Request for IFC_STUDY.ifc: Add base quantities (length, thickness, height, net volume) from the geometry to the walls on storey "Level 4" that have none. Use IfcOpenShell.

First a look at what the model holds.

```python
import ifcopenshell
import ifcopenshell.util.element
import ifcopenshell.util.unit

model = ifcopenshell.open("IFC_STUDY.ifc")
print(model.schema)
for unit_type in ("LENGTHUNIT", "AREAUNIT", "VOLUMEUNIT"):
    print(unit_type, ifcopenshell.util.unit.calculate_unit_scale(model, unit_type))
storey = next(s for s in model.by_type("IfcBuildingStorey") if s.Name == "Level 4")
walls = [e for e in ifcopenshell.util.element.get_decomposition(storey) if e.is_a("IfcWall")]
for e in sorted(walls, key=lambda e: e.id()):
    print(e.id(), e.is_a(), e.Name, list(ifcopenshell.util.element.get_psets(e, qtos_only=True)), sep=" | ")
```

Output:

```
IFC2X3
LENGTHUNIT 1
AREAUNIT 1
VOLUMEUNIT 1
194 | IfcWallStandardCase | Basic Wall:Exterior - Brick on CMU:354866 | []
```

```python
import ifcopenshell
import ifcopenshell.api.pset
import ifcopenshell.geom
import ifcopenshell.util.element
import ifcopenshell.util.shape
import ifcopenshell.util.unit

model = ifcopenshell.open("IFC_STUDY.ifc")
unit_scale = ifcopenshell.util.unit.calculate_unit_scale(model)
volume_scale = ifcopenshell.util.unit.calculate_unit_scale(model, "VOLUMEUNIT")
settings = ifcopenshell.geom.settings()

storey = next(s for s in model.by_type("IfcBuildingStorey") if s.Name == "Level 4")
walls = [e for e in ifcopenshell.util.element.get_decomposition(storey) if e.is_a("IfcWall")]

for e in sorted(walls, key=lambda e: e.id()):
    if ifcopenshell.util.element.get_psets(e, qtos_only=True, should_inherit=False):
        continue
    # Geometry comes back in metres, in the element's own axes.
    shape = ifcopenshell.geom.create_shape(settings, e)
    values = {
        "Length": ifcopenshell.util.shape.get_x(shape.geometry) / unit_scale,
        "Width": ifcopenshell.util.shape.get_y(shape.geometry) / unit_scale,
        "Height": ifcopenshell.util.shape.get_z(shape.geometry) / unit_scale,
        "NetVolume": ifcopenshell.util.shape.get_volume(shape.geometry) / volume_scale,
    }
    qto = ifcopenshell.api.pset.add_qto(model, product=e, name="BaseQuantities")
    ifcopenshell.api.pset.edit_qto(model, qto=qto, properties=values)
    print(e.id(), {k: round(v, 3) for k, v in values.items()})

model.write("IFC_STUDY-out.ifc")
```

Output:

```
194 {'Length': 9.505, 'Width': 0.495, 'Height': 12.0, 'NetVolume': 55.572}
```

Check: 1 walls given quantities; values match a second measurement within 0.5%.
